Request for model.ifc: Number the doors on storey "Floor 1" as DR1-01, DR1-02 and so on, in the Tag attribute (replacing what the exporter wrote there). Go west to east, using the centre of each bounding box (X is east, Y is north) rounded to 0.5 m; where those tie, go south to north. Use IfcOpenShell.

First a look at what the model holds.

```python
import ifcopenshell
import ifcopenshell.util.element
import ifcopenshell.util.placement

model = ifcopenshell.open("model.ifc")
print(model.schema)
storey = next(s for s in model.by_type("IfcBuildingStorey") if s.Name == "Floor 1")
doors = [e for e in ifcopenshell.util.element.get_decomposition(storey) if e.is_a("IfcDoor")]
for e in sorted(doors, key=lambda e: e.id()):
    origin = ifcopenshell.util.placement.get_local_placement(e.ObjectPlacement)[:3, 3]
    print(e.id(), e.Tag, e.Name, origin.round(2) + 0.0, sep=" | ")
```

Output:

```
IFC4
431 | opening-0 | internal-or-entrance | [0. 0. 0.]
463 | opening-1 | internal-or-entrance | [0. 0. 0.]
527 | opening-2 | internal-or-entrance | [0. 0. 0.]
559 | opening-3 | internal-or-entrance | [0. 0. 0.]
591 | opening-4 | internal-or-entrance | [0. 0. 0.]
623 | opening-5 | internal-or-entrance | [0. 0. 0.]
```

```python
import ifcopenshell
import ifcopenshell.geom
import ifcopenshell.util.element
import ifcopenshell.util.shape

model = ifcopenshell.open("model.ifc")
settings = ifcopenshell.geom.settings()
settings.set("use-world-coords", True)


def centre(element):
    shape = ifcopenshell.geom.create_shape(settings, element)
    return ifcopenshell.util.shape.get_bbox_centroid(shape.geometry)


storey = next(s for s in model.by_type("IfcBuildingStorey") if s.Name == "Floor 1")
doors = [e for e in ifcopenshell.util.element.get_decomposition(storey) if e.is_a("IfcDoor")]

# Insertion points can sit at a corner or the storey origin, so sort by the geometry (in metres).
centres = {e: centre(e) for e in doors}
doors.sort(key=lambda e: (round(centres[e][0] / 0.5), centres[e][1]))

for i, e in enumerate(doors, start=1):
    number = f"DR1-{i:02d}"
    e.Tag = number
    print(e.id(), number)

model.write("model_v2.ifc")
```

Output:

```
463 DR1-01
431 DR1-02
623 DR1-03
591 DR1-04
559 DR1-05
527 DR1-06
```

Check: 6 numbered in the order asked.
